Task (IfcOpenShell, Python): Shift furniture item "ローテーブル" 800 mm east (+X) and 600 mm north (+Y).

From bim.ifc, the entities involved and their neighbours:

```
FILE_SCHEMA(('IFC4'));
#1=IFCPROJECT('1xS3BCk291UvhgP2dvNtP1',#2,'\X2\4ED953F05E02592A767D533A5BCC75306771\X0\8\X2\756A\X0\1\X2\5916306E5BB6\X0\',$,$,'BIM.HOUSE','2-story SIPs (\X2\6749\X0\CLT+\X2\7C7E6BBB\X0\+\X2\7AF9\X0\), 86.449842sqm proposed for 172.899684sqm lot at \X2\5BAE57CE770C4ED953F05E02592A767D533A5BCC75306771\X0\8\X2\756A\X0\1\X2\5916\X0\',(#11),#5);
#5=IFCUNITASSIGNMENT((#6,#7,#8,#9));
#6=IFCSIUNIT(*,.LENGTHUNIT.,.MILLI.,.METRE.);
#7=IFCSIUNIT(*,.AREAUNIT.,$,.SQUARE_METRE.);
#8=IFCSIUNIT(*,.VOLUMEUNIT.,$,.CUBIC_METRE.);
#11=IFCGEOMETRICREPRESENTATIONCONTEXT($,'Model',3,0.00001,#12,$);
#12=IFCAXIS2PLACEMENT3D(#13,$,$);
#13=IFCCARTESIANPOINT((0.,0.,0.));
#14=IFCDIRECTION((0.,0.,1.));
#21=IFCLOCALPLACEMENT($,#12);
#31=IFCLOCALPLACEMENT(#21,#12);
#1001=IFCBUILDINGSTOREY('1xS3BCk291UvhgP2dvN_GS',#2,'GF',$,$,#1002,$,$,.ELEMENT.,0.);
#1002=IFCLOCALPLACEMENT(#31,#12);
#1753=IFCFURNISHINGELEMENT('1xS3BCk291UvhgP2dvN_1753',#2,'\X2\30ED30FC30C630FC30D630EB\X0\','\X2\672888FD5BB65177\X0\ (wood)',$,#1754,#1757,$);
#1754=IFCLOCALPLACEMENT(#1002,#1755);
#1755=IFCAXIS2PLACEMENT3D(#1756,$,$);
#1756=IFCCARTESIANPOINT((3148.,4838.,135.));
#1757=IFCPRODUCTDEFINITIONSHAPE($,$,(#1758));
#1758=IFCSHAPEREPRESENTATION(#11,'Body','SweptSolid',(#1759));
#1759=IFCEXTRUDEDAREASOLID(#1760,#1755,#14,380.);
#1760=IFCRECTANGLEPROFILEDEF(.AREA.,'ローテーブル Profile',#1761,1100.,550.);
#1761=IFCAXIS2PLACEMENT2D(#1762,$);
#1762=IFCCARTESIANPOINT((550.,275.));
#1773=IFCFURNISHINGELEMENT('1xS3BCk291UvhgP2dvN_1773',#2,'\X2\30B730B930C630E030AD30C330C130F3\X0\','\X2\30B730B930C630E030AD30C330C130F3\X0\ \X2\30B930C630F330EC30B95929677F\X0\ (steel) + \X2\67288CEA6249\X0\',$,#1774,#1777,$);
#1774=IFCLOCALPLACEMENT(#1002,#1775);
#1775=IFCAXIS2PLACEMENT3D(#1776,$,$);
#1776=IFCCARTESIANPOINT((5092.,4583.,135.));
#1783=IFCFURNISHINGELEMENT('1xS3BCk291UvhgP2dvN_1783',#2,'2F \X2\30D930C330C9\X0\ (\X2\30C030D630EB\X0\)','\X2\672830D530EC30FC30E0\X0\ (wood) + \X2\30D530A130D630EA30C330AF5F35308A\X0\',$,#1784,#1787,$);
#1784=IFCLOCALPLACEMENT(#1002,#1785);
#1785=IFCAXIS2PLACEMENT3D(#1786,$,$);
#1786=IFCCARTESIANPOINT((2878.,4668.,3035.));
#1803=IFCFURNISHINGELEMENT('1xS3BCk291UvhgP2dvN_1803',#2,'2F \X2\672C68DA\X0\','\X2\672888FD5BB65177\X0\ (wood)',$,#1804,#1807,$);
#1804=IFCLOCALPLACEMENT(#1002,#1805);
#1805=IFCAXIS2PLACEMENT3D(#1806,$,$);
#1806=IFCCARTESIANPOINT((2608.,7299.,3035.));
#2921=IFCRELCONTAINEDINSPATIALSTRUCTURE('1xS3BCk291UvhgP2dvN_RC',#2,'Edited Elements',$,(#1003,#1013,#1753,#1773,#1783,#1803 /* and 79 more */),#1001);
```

```python
import ifcopenshell
import ifcopenshell.api.geometry
import ifcopenshell.util.placement
import ifcopenshell.util.unit

model = ifcopenshell.open("bim.ifc")
unit_scale = ifcopenshell.util.unit.calculate_unit_scale(model)

item = model.by_id(1753)
matrix = ifcopenshell.util.placement.get_local_placement(item.ObjectPlacement)
matrix[0, 3] += 0.8 / unit_scale
matrix[1, 3] += 0.6 / unit_scale
ifcopenshell.api.geometry.edit_object_placement(model, product=item, matrix=matrix, is_si=False)

print(ifcopenshell.util.placement.get_local_placement(item.ObjectPlacement).round(3) + 0.0)

model.write("bim_edited.ifc")
```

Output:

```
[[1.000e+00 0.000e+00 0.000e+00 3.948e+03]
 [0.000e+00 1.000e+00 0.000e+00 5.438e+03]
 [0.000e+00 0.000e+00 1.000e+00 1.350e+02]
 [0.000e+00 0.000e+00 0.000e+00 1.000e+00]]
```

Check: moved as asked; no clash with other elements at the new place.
